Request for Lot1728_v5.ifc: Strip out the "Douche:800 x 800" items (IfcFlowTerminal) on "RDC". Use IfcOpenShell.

First a look at what the model holds.

```python
import ifcopenshell
import ifcopenshell.util.element

model = ifcopenshell.open("Lot1728_v5.ifc")
print(model.schema)
storey = next(s for s in model.by_type("IfcBuildingStorey") if s.Name == "RDC")
terminals = [e for e in ifcopenshell.util.element.get_decomposition(storey) if e.is_a("IfcFlowTerminal")]
seen = {}
for e in terminals:
    element_type = ifcopenshell.util.element.get_type(e)
    name = element_type.Name if element_type not in (None, e) else None
    seen[name] = seen.get(name, 0) + 1
for name, count in sorted(seen.items(), key=str):
    print(count, "x", name)
```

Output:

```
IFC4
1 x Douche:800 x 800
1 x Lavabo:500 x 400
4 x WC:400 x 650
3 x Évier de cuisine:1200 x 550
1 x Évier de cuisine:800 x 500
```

```python
import ifcopenshell
import ifcopenshell.api.root
import ifcopenshell.util.element

model = ifcopenshell.open("Lot1728_v5.ifc")

storey = next(s for s in model.by_type("IfcBuildingStorey") if s.Name == "RDC")
terminals = [e for e in ifcopenshell.util.element.get_decomposition(storey) if e.is_a("IfcFlowTerminal")]
targets = [e for e in terminals if (t := ifcopenshell.util.element.get_type(e)) not in (None, e) and t.Name == "Douche:800 x 800"]

for e in targets:
    ifcopenshell.api.root.remove_product(model, product=e)
print(len(targets), "removed")

model.write("Lot1728_v5_v2.ifc")
```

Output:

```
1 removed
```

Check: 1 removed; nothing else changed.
